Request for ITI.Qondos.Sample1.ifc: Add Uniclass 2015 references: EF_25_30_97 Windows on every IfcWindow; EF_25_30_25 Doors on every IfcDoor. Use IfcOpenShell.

First a look at what the model holds.

```python
import ifcopenshell

model = ifcopenshell.open("ITI.Qondos.Sample1.ifc")
print(model.schema)
print("classifications:", [c.Name for c in model.by_type("IfcClassification")])
for ifc_class in ("IfcDoor", "IfcRoof", "IfcStair", "IfcWall", "IfcWindow"):
    print(ifc_class, len(model.by_type(ifc_class)))
```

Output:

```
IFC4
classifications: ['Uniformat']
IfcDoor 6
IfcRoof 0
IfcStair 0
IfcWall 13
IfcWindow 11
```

```python
import ifcopenshell
import ifcopenshell.api.classification

model = ifcopenshell.open("ITI.Qondos.Sample1.ifc")

system = ifcopenshell.api.classification.add_classification(model, classification="Uniclass 2015")

codes = {
    "IfcWindow": ("EF_25_30_97", "Windows"),
    "IfcDoor": ("EF_25_30_25", "Doors"),
}
for ifc_class, (code, name) in codes.items():
    products = model.by_type(ifc_class)
    ifcopenshell.api.classification.add_reference(
        model, products=products, classification=system, identification=code, name=name
    )
    print(code, len(products))

model.write("ITI.Qondos.Sample1_v2.ifc")
```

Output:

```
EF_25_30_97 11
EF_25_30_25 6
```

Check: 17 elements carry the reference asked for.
